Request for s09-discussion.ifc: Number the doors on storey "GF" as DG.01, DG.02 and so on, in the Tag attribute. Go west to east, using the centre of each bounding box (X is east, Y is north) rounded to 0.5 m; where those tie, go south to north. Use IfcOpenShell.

First a look at what the model holds.

```python
import ifcopenshell
import ifcopenshell.util.element
import ifcopenshell.util.placement

model = ifcopenshell.open("s09-discussion.ifc")
print(model.schema)
storey = next(s for s in model.by_type("IfcBuildingStorey") if s.Name == "GF")
doors = [e for e in ifcopenshell.util.element.get_decomposition(storey) if e.is_a("IfcDoor")]
for e in sorted(doors, key=lambda e: e.id()):
    origin = ifcopenshell.util.placement.get_local_placement(e.ObjectPlacement)[:3, 3]
    print(e.id(), e.Tag, e.Name, origin.round(2) + 0.0, sep=" | ")
```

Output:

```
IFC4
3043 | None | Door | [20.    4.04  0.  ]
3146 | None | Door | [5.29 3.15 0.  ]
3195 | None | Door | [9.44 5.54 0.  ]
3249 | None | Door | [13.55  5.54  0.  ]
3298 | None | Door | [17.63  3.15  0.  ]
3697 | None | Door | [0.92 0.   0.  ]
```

```python
import ifcopenshell
import ifcopenshell.geom
import ifcopenshell.util.element
import ifcopenshell.util.shape

model = ifcopenshell.open("s09-discussion.ifc")
settings = ifcopenshell.geom.settings()
settings.set("use-world-coords", True)


def centre(element):
    shape = ifcopenshell.geom.create_shape(settings, element)
    return ifcopenshell.util.shape.get_bbox_centroid(shape.geometry)


storey = next(s for s in model.by_type("IfcBuildingStorey") if s.Name == "GF")
doors = [e for e in ifcopenshell.util.element.get_decomposition(storey) if e.is_a("IfcDoor")]

# Insertion points can sit at a corner or the storey origin, so sort by the geometry (in metres).
centres = {e: centre(e) for e in doors}
doors.sort(key=lambda e: (round(centres[e][0] / 0.5), centres[e][1]))

for i, e in enumerate(doors, start=1):
    number = f"DG.{i:02d}"
    e.Tag = number
    print(e.id(), number)

model.write("s09-discussion_edited.ifc")
```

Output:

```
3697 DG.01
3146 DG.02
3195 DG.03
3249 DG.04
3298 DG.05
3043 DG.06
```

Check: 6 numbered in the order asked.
